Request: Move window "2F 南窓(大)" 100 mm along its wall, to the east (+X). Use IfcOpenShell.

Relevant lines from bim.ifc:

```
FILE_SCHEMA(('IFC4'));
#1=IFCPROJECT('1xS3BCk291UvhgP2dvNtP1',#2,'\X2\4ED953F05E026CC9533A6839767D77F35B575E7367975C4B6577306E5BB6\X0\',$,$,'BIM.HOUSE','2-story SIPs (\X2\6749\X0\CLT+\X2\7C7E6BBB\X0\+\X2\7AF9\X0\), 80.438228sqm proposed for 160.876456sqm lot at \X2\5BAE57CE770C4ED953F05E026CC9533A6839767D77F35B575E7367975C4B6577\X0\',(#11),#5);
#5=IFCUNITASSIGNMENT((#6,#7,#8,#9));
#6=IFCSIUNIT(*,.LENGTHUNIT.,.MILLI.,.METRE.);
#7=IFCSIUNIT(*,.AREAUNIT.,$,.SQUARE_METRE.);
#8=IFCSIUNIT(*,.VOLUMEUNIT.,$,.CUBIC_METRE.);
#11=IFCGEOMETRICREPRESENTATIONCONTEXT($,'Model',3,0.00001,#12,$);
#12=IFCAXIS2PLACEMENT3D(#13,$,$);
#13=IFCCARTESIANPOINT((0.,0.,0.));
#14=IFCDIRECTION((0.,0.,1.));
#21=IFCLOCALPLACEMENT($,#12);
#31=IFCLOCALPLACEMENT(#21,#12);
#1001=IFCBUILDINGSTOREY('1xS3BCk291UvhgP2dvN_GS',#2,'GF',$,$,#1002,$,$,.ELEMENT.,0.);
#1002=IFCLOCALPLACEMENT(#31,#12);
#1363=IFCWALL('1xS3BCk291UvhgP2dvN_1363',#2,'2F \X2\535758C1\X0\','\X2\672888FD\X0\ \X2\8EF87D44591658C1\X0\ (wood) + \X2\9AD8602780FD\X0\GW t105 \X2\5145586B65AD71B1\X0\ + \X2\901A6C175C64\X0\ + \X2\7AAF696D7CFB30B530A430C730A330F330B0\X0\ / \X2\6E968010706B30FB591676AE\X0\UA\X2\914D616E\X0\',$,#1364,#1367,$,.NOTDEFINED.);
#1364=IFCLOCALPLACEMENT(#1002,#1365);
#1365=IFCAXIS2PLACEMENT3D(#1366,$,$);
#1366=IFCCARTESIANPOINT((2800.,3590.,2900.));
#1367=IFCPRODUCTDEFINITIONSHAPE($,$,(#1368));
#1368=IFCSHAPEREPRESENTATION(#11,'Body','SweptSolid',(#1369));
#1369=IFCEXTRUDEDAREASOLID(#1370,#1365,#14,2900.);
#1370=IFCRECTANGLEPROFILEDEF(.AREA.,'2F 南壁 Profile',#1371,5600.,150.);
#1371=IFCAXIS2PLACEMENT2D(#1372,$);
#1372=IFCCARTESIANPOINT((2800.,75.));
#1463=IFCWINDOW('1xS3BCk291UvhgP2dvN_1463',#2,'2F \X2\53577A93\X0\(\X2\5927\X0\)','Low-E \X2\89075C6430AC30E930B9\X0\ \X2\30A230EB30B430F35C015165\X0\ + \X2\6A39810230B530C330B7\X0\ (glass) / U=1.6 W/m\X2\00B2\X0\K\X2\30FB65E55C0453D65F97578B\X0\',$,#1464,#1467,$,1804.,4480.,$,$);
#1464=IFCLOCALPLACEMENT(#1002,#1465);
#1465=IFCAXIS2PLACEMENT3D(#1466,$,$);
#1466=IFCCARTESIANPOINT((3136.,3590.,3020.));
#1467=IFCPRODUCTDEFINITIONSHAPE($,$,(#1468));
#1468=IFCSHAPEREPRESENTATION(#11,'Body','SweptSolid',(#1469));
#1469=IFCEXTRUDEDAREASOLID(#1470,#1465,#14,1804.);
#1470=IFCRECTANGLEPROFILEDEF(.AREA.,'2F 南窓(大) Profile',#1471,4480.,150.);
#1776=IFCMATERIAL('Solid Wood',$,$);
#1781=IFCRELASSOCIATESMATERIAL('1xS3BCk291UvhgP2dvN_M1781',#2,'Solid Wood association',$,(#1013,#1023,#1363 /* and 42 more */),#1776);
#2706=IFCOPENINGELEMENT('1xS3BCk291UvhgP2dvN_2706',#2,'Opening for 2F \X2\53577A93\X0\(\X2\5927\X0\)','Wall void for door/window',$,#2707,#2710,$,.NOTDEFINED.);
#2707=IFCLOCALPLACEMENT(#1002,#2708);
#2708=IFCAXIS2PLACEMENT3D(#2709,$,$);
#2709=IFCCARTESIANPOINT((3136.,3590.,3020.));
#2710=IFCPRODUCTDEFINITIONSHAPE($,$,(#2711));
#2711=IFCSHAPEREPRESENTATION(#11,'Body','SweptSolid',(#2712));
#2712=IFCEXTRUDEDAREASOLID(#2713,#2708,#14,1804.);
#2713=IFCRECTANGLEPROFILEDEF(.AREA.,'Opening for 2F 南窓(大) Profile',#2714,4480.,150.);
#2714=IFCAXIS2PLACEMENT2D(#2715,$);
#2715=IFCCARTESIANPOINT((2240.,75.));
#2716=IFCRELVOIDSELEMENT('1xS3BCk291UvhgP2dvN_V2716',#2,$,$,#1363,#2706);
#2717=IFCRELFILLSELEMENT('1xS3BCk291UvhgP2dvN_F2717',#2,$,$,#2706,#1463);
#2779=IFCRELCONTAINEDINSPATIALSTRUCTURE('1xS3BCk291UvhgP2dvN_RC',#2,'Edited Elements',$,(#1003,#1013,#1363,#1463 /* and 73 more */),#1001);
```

```python
import ifcopenshell
import ifcopenshell.api.geometry
import ifcopenshell.util.placement

model = ifcopenshell.open("bim.ifc")

window = model.by_id(1463)
opening = window.FillsVoids[0].RelatingOpeningElement
wall = opening.VoidsElements[0].RelatingBuildingElement

wall_matrix = ifcopenshell.util.placement.get_local_placement(wall.ObjectPlacement)
shift = wall_matrix[:3, 0] * 100.0
before = ifcopenshell.util.placement.get_local_placement(window.ObjectPlacement)[:3, 3].copy()

# The window is not placed relative to its opening, so move both.
for product in (opening, window):
    matrix = ifcopenshell.util.placement.get_local_placement(product.ObjectPlacement)
    matrix[:3, 3] += shift
    ifcopenshell.api.geometry.edit_object_placement(model, product=product, matrix=matrix, is_si=False)

after = ifcopenshell.util.placement.get_local_placement(window.ObjectPlacement)[:3, 3]
print("window moved by", (after - before).round(3) + 0.0)

model.write("bim_edited.ifc")
```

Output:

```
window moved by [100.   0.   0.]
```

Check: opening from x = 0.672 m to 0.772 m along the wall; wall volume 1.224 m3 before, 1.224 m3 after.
